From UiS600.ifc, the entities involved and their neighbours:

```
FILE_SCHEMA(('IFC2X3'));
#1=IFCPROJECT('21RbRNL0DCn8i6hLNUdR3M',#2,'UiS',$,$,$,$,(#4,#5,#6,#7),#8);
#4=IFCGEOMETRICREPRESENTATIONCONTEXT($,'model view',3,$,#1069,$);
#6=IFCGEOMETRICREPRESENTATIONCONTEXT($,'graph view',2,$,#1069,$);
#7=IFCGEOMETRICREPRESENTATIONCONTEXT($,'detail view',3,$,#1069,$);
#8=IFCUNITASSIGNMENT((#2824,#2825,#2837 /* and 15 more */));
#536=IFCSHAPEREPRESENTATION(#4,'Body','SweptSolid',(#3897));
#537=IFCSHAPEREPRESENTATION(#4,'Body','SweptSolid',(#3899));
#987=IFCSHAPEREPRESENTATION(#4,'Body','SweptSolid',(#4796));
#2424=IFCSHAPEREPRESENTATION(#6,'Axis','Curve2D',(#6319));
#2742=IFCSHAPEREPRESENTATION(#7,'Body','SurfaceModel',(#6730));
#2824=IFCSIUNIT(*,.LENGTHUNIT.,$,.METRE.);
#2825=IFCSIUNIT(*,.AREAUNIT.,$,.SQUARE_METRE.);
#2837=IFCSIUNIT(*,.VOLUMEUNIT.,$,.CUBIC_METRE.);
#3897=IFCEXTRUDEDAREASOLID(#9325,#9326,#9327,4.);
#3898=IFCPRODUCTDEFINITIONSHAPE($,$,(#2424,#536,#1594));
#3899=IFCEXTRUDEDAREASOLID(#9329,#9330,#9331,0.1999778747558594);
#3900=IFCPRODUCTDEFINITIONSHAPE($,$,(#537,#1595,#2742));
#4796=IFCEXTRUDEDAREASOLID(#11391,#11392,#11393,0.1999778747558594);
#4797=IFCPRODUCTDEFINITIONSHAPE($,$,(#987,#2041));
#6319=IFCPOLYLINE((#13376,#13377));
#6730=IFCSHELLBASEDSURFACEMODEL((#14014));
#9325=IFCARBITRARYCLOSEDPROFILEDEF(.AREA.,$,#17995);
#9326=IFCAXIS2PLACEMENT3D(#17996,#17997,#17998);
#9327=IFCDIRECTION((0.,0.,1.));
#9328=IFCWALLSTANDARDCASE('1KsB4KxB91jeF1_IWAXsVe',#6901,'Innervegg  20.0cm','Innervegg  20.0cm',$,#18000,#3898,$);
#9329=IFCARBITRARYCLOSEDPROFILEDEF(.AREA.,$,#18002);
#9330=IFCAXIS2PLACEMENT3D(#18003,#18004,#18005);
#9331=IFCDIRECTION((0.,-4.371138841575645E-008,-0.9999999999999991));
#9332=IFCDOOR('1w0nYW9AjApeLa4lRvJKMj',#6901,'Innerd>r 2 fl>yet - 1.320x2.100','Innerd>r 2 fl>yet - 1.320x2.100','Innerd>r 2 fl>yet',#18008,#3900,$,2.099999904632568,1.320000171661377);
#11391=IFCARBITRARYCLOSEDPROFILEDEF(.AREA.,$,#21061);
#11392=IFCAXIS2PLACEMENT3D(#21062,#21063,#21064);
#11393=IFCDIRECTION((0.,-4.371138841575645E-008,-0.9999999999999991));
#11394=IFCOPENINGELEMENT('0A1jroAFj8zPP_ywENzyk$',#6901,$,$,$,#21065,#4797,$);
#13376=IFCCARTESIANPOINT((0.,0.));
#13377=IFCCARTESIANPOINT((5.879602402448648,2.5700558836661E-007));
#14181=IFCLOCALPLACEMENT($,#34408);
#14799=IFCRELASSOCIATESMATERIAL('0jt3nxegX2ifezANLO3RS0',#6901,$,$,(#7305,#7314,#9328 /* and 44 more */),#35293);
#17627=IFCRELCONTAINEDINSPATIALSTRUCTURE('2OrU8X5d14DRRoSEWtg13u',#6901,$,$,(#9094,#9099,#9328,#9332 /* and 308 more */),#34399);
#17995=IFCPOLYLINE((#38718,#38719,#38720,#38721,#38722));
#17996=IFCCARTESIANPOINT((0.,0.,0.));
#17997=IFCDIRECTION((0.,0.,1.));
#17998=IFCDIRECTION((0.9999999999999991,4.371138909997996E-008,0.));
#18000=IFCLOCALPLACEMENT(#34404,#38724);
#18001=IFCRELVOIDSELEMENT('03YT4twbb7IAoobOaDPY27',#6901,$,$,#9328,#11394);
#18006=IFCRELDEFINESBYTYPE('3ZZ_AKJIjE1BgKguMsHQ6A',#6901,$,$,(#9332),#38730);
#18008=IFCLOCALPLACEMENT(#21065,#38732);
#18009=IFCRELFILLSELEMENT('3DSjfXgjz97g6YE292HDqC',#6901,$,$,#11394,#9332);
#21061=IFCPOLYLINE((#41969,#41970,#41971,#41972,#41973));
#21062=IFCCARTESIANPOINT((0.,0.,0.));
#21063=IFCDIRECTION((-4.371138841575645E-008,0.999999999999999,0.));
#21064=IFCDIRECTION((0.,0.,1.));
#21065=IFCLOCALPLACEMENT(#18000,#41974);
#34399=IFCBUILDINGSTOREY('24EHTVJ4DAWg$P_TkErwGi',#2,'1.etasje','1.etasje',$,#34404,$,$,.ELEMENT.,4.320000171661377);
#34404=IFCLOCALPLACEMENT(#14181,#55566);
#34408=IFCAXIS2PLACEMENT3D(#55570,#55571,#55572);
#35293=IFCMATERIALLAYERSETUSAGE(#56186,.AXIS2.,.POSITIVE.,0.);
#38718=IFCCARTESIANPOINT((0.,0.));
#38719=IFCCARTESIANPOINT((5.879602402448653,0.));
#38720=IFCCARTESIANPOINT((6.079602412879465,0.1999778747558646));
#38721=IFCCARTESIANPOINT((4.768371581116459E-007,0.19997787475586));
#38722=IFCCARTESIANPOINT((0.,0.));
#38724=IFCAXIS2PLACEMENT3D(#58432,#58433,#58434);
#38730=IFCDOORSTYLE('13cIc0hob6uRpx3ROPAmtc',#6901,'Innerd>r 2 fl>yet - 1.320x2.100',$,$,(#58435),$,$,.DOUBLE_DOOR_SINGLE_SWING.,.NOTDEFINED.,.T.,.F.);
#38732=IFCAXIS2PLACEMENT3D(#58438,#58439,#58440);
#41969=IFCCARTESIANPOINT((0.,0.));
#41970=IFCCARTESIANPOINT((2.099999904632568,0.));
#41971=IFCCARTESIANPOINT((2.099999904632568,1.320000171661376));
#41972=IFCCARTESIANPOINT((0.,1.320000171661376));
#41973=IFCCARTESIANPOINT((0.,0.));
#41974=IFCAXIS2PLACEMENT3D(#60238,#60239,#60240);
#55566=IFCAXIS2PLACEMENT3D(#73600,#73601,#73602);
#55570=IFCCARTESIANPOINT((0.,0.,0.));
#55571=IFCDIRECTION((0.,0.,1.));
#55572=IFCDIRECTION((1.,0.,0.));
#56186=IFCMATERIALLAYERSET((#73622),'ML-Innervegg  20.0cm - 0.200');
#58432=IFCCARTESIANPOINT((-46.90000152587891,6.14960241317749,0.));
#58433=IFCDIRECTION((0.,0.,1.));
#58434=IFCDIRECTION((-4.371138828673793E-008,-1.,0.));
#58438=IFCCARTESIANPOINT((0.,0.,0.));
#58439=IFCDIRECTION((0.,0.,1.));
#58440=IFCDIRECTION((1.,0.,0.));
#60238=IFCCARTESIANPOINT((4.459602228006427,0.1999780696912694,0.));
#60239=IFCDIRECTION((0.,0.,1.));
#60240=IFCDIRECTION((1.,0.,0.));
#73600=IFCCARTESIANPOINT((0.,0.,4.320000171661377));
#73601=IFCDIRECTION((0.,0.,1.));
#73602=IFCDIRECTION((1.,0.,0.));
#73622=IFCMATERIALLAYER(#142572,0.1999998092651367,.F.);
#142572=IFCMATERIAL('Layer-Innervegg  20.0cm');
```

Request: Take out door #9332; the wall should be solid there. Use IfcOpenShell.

```python
import ifcopenshell
import ifcopenshell.api.feature
import ifcopenshell.api.root
import ifcopenshell.geom
import ifcopenshell.util.shape

model = ifcopenshell.open("UiS600.ifc")
settings = ifcopenshell.geom.settings()


def volume(element):
    """Net volume in cubic metres, openings subtracted."""
    shape = ifcopenshell.geom.create_shape(settings, element)
    return ifcopenshell.util.shape.get_volume(shape.geometry)


door = model.by_guid("1w0nYW9AjApeLa4lRvJKMj")
opening = door.FillsVoids[0].RelatingOpeningElement
wall = opening.VoidsElements[0].RelatingBuildingElement
before = volume(wall)

ifcopenshell.api.root.remove_product(model, product=door)
ifcopenshell.api.feature.remove_feature(model, feature=opening)

after = volume(wall)

print(f"wall volume {before:.3f} -> {after:.3f} m3")

model.write("UiS600_updated.ifc")
```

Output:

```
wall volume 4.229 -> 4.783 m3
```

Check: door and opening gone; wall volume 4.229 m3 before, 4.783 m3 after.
